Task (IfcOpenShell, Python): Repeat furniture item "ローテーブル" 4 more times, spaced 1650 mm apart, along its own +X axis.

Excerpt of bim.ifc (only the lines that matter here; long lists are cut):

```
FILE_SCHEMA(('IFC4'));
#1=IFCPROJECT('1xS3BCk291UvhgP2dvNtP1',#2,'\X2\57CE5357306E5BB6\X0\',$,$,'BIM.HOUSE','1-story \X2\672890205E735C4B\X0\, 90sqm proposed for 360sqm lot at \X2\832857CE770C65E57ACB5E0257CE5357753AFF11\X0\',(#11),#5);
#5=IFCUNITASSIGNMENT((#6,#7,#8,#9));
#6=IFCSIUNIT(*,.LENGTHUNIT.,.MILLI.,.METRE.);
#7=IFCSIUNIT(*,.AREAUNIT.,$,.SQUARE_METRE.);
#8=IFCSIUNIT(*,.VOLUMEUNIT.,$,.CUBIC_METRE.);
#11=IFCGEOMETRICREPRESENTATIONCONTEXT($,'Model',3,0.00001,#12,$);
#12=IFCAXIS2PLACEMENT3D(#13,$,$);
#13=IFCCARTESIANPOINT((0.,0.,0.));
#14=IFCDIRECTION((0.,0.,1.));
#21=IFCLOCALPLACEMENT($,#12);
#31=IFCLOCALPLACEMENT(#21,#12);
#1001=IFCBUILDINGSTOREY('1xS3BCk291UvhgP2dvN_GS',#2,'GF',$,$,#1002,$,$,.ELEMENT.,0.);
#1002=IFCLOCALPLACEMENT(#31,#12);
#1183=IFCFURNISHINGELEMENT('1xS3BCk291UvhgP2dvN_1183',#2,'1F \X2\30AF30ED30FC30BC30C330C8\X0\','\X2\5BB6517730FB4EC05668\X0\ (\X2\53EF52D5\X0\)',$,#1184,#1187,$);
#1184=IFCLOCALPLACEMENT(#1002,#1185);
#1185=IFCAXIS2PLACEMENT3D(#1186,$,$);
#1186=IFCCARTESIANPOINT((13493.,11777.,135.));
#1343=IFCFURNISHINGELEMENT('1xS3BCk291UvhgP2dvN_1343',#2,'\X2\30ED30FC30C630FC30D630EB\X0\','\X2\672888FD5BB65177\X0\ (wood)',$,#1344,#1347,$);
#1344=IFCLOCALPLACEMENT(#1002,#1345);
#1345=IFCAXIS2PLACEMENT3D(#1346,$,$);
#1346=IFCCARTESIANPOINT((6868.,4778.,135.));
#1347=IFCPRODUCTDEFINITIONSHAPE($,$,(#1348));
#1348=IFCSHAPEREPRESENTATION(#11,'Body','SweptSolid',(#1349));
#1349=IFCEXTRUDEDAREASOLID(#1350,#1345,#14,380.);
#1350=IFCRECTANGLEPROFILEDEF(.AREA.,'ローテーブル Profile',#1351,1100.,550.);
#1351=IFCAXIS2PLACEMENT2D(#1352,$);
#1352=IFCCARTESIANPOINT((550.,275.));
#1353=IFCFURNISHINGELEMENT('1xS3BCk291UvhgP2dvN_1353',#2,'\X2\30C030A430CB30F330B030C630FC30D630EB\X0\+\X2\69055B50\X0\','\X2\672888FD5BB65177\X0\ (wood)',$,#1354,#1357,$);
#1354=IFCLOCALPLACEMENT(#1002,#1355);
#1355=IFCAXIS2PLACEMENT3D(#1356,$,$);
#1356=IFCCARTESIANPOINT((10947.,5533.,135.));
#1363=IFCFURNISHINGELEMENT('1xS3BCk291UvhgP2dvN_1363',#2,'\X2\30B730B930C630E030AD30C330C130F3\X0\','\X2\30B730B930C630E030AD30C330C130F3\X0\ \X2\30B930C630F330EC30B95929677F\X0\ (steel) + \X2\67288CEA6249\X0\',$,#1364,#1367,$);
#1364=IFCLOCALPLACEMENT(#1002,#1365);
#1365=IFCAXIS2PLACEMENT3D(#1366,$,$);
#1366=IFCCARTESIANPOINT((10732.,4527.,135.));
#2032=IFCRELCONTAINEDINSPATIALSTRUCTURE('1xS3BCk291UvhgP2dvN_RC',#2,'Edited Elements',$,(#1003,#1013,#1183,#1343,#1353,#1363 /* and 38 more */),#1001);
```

```python
import ifcopenshell
import ifcopenshell.api.geometry
import ifcopenshell.api.root
import ifcopenshell.util.element
import ifcopenshell.util.placement

model = ifcopenshell.open("bim.ifc")


def reuse_history(source, copy):
    """copy_class also copies each property set's owner history, people and application; keep the originals."""
    for rel in copy.IsDefinedBy:
        if rel.is_a("IfcRelDefinesByProperties") and (history := rel.RelatingPropertyDefinition.OwnerHistory):
            rel.RelatingPropertyDefinition.OwnerHistory = source.OwnerHistory
            ifcopenshell.util.element.remove_deep2(model, history)


source = model.by_guid("1xS3BCk291UvhgP2dvN_1343")
base = ifcopenshell.util.placement.get_local_placement(source.ObjectPlacement)
step = base[:3, 0] * 1650.0

for i in range(1, 5):
    copy = ifcopenshell.api.root.copy_class(model, product=source)
    copy.Representation = ifcopenshell.util.element.copy_deep(
        model, source.Representation, exclude=["IfcGeometricRepresentationContext", "IfcRepresentationMap"]
    )
    reuse_history(source, copy)
    matrix = base.copy()
    matrix[:3, 3] += i * step
    print("added at", matrix[:3, 3].round(3) + 0.0)
    ifcopenshell.api.geometry.edit_object_placement(model, product=copy, matrix=matrix, is_si=False)

model.write("bim_rev.ifc")
```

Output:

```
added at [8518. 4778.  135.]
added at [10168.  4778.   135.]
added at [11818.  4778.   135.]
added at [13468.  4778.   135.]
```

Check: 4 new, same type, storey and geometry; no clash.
